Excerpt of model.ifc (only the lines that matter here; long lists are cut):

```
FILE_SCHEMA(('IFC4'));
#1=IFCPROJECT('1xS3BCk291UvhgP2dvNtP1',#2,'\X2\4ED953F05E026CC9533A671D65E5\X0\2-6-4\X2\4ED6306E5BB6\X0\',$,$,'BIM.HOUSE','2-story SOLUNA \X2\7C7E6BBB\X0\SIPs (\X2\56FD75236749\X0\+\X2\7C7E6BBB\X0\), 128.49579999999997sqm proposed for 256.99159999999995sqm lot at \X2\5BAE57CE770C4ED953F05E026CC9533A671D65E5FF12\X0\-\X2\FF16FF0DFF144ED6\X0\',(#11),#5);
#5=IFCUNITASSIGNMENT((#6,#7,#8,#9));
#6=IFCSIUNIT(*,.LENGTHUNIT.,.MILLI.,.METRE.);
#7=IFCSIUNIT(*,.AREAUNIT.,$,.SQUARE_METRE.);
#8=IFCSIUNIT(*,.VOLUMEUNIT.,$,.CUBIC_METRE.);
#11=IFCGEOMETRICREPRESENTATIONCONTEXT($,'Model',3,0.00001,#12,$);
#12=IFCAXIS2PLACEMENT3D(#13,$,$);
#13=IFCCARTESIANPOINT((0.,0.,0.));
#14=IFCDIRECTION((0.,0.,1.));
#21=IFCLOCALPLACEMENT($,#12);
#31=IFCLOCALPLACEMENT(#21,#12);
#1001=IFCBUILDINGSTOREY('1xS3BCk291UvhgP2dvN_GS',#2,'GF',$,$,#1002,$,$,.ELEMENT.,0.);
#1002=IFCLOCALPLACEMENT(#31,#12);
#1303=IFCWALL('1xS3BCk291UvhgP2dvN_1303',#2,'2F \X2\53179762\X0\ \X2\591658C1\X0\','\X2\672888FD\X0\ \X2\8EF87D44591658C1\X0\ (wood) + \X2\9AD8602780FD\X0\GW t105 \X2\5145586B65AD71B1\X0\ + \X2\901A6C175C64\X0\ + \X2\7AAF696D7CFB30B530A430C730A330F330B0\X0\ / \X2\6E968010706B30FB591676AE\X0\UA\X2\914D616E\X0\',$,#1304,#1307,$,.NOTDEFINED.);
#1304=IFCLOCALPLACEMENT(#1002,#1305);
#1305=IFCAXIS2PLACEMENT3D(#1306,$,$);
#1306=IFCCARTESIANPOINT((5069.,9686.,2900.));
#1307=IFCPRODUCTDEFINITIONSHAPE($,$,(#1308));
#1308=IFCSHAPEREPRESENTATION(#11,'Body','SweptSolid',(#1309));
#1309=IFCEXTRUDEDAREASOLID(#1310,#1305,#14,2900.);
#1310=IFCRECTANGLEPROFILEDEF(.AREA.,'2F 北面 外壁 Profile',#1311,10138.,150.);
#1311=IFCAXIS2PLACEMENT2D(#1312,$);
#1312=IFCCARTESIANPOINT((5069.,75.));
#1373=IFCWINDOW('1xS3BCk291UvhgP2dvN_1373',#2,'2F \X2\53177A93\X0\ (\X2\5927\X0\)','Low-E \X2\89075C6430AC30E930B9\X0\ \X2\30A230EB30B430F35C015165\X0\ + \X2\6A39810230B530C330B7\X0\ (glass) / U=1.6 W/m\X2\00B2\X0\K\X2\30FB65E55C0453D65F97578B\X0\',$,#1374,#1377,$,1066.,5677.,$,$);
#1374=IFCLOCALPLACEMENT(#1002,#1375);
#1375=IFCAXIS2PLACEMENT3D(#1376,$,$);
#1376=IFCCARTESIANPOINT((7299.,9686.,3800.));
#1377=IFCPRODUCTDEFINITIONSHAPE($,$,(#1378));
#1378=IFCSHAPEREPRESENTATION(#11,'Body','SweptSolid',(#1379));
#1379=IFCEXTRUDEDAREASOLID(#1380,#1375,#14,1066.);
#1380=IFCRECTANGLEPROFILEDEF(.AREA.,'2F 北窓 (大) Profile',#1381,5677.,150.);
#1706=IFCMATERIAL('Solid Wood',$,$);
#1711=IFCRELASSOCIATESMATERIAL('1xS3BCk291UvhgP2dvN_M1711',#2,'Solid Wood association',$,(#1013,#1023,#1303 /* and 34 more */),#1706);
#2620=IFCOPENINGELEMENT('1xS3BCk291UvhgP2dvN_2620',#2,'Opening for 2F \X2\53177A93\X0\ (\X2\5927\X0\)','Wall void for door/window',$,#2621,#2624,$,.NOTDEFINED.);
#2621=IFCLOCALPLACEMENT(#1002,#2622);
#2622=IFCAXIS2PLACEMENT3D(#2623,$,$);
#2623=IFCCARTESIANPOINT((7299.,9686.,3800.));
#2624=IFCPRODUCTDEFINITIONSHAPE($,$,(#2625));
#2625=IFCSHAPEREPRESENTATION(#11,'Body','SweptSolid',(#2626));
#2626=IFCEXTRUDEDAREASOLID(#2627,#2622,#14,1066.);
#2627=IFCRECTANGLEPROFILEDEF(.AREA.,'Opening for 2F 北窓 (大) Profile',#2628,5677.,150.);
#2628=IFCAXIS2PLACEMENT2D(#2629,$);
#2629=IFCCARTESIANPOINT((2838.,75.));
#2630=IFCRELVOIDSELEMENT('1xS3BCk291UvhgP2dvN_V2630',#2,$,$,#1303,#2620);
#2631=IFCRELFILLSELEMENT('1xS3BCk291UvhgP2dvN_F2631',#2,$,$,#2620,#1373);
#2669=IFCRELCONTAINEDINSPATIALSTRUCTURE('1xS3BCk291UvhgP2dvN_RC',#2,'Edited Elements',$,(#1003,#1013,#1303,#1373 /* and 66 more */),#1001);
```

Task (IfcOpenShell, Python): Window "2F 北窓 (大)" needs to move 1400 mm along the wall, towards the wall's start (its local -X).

```python
import ifcopenshell
import ifcopenshell.api.geometry
import ifcopenshell.util.placement
import ifcopenshell.util.unit

model = ifcopenshell.open("model.ifc")
unit_scale = ifcopenshell.util.unit.calculate_unit_scale(model)

window = model.by_guid("1xS3BCk291UvhgP2dvN_1373")
opening = window.FillsVoids[0].RelatingOpeningElement
wall = opening.VoidsElements[0].RelatingBuildingElement

wall_matrix = ifcopenshell.util.placement.get_local_placement(wall.ObjectPlacement)
shift = wall_matrix[:3, 0] * -1.4 / unit_scale
before = ifcopenshell.util.placement.get_local_placement(window.ObjectPlacement)[:3, 3].copy()

# The window is not placed relative to its opening, so move both.
for product in (opening, window):
    matrix = ifcopenshell.util.placement.get_local_placement(product.ObjectPlacement)
    matrix[:3, 3] += shift
    ifcopenshell.api.geometry.edit_object_placement(model, product=product, matrix=matrix, is_si=False)

after = ifcopenshell.util.placement.get_local_placement(window.ObjectPlacement)[:3, 3]
print("window moved by", (after - before).round(3) + 0.0)

model.write("model_edited.ifc")
```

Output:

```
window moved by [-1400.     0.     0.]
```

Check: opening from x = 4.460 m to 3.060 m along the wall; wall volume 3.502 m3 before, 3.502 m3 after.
